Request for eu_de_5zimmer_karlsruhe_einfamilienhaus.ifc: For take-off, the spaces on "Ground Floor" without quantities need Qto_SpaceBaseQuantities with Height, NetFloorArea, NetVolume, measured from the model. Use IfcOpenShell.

First a look at what the model holds.

```python
import ifcopenshell
import ifcopenshell.util.element
import ifcopenshell.util.unit

model = ifcopenshell.open("eu_de_5zimmer_karlsruhe_einfamilienhaus.ifc")
print(model.schema)
for unit_type in ("LENGTHUNIT", "AREAUNIT", "VOLUMEUNIT"):
    print(unit_type, ifcopenshell.util.unit.calculate_unit_scale(model, unit_type))
storey = next(s for s in model.by_type("IfcBuildingStorey") if s.Name == "Ground Floor")
spaces = [e for e in ifcopenshell.util.element.get_decomposition(storey) if e.is_a("IfcSpace")]
for e in sorted(spaces, key=lambda e: e.id()):
    print(e.id(), e.is_a(), e.Name, list(ifcopenshell.util.element.get_psets(e, qtos_only=True)), sep=" | ")
```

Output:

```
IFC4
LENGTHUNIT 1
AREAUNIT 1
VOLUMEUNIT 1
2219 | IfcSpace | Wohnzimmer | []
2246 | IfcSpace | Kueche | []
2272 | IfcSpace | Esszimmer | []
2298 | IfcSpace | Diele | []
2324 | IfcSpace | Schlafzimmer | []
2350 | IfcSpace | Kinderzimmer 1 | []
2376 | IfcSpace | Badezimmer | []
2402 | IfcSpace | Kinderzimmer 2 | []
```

```python
import ifcopenshell
import ifcopenshell.api.pset
import ifcopenshell.geom
import ifcopenshell.util.element
import ifcopenshell.util.shape
import ifcopenshell.util.unit

model = ifcopenshell.open("eu_de_5zimmer_karlsruhe_einfamilienhaus.ifc")
unit_scale = ifcopenshell.util.unit.calculate_unit_scale(model)
area_scale = ifcopenshell.util.unit.calculate_unit_scale(model, "AREAUNIT")
volume_scale = ifcopenshell.util.unit.calculate_unit_scale(model, "VOLUMEUNIT")
settings = ifcopenshell.geom.settings()

storey = next(s for s in model.by_type("IfcBuildingStorey") if s.Name == "Ground Floor")
spaces = [e for e in ifcopenshell.util.element.get_decomposition(storey) if e.is_a("IfcSpace")]

for e in sorted(spaces, key=lambda e: e.id()):
    if ifcopenshell.util.element.get_psets(e, qtos_only=True, should_inherit=False):
        continue
    # Geometry comes back in metres, in the element's own axes.
    shape = ifcopenshell.geom.create_shape(settings, e)
    values = {
        "Height": ifcopenshell.util.shape.get_z(shape.geometry) / unit_scale,
        "NetFloorArea": ifcopenshell.util.shape.get_footprint_area(shape.geometry) / area_scale,
        "NetVolume": ifcopenshell.util.shape.get_volume(shape.geometry) / volume_scale,
    }
    qto = ifcopenshell.api.pset.add_qto(model, product=e, name="Qto_SpaceBaseQuantities")
    ifcopenshell.api.pset.edit_qto(model, qto=qto, properties=values)
    print(e.id(), {k: round(v, 3) for k, v in values.items()})

model.write("eu_de_5zimmer_karlsruhe_einfamilienhaus_updated.ifc")
```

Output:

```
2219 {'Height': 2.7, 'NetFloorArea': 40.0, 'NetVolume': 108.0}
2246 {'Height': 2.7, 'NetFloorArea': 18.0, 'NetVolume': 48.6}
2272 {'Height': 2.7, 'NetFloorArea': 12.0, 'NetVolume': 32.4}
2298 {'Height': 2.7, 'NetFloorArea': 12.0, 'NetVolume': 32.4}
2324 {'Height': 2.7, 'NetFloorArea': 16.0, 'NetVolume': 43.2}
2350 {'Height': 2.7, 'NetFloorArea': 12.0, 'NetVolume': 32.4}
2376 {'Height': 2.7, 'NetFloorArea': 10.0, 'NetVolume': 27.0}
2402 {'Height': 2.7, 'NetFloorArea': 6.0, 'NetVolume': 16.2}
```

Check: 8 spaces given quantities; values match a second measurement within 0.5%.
